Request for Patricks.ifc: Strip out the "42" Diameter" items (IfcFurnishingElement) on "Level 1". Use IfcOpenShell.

First a look at what the model holds.

```python
import ifcopenshell
import ifcopenshell.util.element

model = ifcopenshell.open("Patricks.ifc")
print(model.schema)
storey = next(s for s in model.by_type("IfcBuildingStorey") if s.Name == "Level 1")
furniture = [e for e in ifcopenshell.util.element.get_decomposition(storey) if e.is_a("IfcFurnishingElement")]
seen = {}
for e in furniture:
    element_type = ifcopenshell.util.element.get_type(e)
    name = element_type.Name if element_type not in (None, e) else None
    seen[name] = seen.get(name, 0) + 1
for name, count in sorted(seen.items(), key=str):
    print(count, "x", name)
```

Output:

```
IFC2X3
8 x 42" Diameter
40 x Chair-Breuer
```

```python
import ifcopenshell
import ifcopenshell.api.root
import ifcopenshell.util.element

model = ifcopenshell.open("Patricks.ifc")

storey = next(s for s in model.by_type("IfcBuildingStorey") if s.Name == "Level 1")
furniture = [e for e in ifcopenshell.util.element.get_decomposition(storey) if e.is_a("IfcFurnishingElement")]
targets = [e for e in furniture if (t := ifcopenshell.util.element.get_type(e)) not in (None, e) and t.Name == '42" Diameter']

for e in targets:
    ifcopenshell.api.root.remove_product(model, product=e)
print(len(targets), "removed")

model.write("Patricks_v2.ifc")
```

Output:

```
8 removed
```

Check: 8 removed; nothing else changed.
